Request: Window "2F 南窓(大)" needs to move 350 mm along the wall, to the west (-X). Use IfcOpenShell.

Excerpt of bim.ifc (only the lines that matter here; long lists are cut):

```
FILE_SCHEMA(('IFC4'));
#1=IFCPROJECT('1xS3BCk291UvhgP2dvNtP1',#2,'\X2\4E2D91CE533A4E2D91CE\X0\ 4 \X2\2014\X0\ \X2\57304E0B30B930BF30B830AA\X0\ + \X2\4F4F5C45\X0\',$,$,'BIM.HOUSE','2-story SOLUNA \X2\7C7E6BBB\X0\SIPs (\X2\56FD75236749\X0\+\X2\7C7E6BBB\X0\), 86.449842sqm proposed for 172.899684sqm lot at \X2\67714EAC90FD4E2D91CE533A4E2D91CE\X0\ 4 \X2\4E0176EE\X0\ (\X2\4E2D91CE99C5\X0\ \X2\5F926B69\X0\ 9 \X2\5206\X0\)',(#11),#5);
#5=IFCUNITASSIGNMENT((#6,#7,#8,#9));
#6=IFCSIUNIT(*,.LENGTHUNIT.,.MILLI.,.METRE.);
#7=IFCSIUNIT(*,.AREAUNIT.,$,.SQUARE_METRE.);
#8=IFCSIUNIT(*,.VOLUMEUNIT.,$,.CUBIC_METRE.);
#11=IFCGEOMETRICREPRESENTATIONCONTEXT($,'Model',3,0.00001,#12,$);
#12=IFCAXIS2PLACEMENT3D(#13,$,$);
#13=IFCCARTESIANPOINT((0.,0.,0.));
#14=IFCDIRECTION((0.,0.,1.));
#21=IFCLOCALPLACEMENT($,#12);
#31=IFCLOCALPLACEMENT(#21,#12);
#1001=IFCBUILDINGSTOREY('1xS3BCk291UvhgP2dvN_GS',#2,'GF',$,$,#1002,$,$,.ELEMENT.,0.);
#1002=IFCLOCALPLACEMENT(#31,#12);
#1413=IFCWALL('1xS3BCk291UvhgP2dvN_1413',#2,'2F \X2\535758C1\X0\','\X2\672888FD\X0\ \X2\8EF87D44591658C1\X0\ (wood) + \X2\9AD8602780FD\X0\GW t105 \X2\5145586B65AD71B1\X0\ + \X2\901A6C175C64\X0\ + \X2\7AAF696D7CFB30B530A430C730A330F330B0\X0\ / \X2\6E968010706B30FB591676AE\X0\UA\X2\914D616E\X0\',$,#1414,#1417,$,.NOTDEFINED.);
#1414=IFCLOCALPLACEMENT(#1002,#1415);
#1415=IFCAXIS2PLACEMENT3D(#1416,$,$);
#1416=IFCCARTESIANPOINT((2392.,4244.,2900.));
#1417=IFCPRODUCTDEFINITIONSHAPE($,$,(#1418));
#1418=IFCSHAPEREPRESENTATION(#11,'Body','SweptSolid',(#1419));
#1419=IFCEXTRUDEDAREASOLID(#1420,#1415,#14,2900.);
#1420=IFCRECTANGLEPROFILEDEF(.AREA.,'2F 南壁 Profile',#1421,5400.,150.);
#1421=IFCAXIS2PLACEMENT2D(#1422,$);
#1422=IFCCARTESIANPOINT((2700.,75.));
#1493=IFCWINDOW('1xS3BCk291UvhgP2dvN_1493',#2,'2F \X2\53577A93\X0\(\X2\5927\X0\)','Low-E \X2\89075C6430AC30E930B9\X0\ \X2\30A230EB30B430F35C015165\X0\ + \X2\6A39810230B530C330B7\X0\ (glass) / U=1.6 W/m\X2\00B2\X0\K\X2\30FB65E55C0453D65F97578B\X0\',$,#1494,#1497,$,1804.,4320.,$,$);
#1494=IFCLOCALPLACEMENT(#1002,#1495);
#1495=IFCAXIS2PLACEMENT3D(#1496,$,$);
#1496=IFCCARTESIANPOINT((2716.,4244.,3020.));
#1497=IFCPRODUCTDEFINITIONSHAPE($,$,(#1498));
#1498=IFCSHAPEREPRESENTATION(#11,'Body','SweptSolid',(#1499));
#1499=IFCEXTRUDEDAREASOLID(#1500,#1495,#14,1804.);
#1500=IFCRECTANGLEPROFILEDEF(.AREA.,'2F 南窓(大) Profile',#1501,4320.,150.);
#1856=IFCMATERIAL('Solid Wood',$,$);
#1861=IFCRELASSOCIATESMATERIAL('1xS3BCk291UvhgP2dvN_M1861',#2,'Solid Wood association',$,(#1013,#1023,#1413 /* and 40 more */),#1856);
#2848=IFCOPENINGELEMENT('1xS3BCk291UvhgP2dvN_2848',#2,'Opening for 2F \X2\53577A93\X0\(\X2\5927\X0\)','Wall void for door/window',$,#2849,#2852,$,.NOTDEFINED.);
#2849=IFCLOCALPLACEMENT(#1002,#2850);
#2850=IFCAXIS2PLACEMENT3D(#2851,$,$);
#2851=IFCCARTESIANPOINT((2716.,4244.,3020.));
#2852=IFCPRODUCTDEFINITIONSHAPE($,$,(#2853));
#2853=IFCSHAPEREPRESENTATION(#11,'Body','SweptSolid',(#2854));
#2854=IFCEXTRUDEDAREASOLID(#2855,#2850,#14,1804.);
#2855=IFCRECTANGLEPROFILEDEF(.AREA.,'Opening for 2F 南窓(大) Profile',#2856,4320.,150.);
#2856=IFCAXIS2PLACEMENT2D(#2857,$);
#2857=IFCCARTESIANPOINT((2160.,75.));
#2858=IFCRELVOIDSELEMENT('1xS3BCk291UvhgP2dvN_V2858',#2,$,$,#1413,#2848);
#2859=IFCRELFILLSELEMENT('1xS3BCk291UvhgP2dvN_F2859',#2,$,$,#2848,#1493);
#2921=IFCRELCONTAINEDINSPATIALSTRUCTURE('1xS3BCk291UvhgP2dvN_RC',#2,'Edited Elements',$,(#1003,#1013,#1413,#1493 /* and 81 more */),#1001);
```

```python
import ifcopenshell
import ifcopenshell.api.geometry
import ifcopenshell.util.placement
import ifcopenshell.util.unit

model = ifcopenshell.open("bim.ifc")
unit_scale = ifcopenshell.util.unit.calculate_unit_scale(model)

window = model.by_guid("1xS3BCk291UvhgP2dvN_1493")
opening = window.FillsVoids[0].RelatingOpeningElement
wall = opening.VoidsElements[0].RelatingBuildingElement

wall_matrix = ifcopenshell.util.placement.get_local_placement(wall.ObjectPlacement)
shift = wall_matrix[:3, 0] * -0.35 / unit_scale
before = ifcopenshell.util.placement.get_local_placement(window.ObjectPlacement)[:3, 3].copy()

# The window is not placed relative to its opening, so move both.
for product in (opening, window):
    matrix = ifcopenshell.util.placement.get_local_placement(product.ObjectPlacement)
    matrix[:3, 3] += shift
    ifcopenshell.api.geometry.edit_object_placement(model, product=product, matrix=matrix, is_si=False)

after = ifcopenshell.util.placement.get_local_placement(window.ObjectPlacement)[:3, 3]
print("window moved by", (after - before).round(3) + 0.0)

model.write("bim-out.ifc")
```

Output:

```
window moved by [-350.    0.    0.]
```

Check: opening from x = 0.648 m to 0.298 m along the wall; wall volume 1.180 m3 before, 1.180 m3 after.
